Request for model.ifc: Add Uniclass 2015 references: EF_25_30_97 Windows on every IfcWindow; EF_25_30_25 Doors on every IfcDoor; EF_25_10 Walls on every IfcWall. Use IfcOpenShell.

First a look at what the model holds.

```python
import ifcopenshell

model = ifcopenshell.open("model.ifc")
print(model.schema)
print("classifications:", [c.Name for c in model.by_type("IfcClassification")])
for ifc_class in ("IfcDoor", "IfcRoof", "IfcStair", "IfcWall", "IfcWindow"):
    print(ifc_class, len(model.by_type(ifc_class)))
```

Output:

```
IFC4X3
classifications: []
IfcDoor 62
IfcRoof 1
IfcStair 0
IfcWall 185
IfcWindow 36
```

```python
import ifcopenshell
import ifcopenshell.api.classification

model = ifcopenshell.open("model.ifc")

system = ifcopenshell.api.classification.add_classification(model, classification="Uniclass 2015")

codes = {
    "IfcWindow": ("EF_25_30_97", "Windows"),
    "IfcDoor": ("EF_25_30_25", "Doors"),
    "IfcWall": ("EF_25_10", "Walls"),
}
for ifc_class, (code, name) in codes.items():
    products = model.by_type(ifc_class)
    ifcopenshell.api.classification.add_reference(
        model, products=products, classification=system, identification=code, name=name
    )
    print(code, len(products))

model.write("model-out.ifc")
```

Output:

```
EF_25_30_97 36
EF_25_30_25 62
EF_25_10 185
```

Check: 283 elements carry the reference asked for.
